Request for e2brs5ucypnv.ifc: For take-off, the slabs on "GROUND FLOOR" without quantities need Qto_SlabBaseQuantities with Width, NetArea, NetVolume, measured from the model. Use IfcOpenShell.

First a look at what the model holds.

```python
import ifcopenshell
import ifcopenshell.util.element
import ifcopenshell.util.unit

model = ifcopenshell.open("e2brs5ucypnv.ifc")
print(model.schema)
for unit_type in ("LENGTHUNIT", "AREAUNIT", "VOLUMEUNIT"):
    print(unit_type, ifcopenshell.util.unit.calculate_unit_scale(model, unit_type))
storey = next(s for s in model.by_type("IfcBuildingStorey") if s.Name == "GROUND FLOOR")
slabs = [e for e in ifcopenshell.util.element.get_decomposition(storey) if e.is_a("IfcSlab")]
for e in sorted(slabs, key=lambda e: e.id()):
    print(e.id(), e.is_a(), e.Name, list(ifcopenshell.util.element.get_psets(e, qtos_only=True)), sep=" | ")
```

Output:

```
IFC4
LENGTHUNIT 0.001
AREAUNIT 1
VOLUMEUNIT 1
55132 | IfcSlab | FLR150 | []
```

```python
import ifcopenshell
import ifcopenshell.api.pset
import ifcopenshell.geom
import ifcopenshell.util.element
import ifcopenshell.util.shape
import ifcopenshell.util.unit

model = ifcopenshell.open("e2brs5ucypnv.ifc")
unit_scale = ifcopenshell.util.unit.calculate_unit_scale(model)
area_scale = ifcopenshell.util.unit.calculate_unit_scale(model, "AREAUNIT")
volume_scale = ifcopenshell.util.unit.calculate_unit_scale(model, "VOLUMEUNIT")
settings = ifcopenshell.geom.settings()

storey = next(s for s in model.by_type("IfcBuildingStorey") if s.Name == "GROUND FLOOR")
slabs = [e for e in ifcopenshell.util.element.get_decomposition(storey) if e.is_a("IfcSlab")]

for e in sorted(slabs, key=lambda e: e.id()):
    if ifcopenshell.util.element.get_psets(e, qtos_only=True, should_inherit=False):
        continue
    # Geometry comes back in metres, in the element's own axes.
    shape = ifcopenshell.geom.create_shape(settings, e)
    values = {
        "Width": ifcopenshell.util.shape.get_z(shape.geometry) / unit_scale,
        "NetArea": ifcopenshell.util.shape.get_footprint_area(shape.geometry) / area_scale,
        "NetVolume": ifcopenshell.util.shape.get_volume(shape.geometry) / volume_scale,
    }
    qto = ifcopenshell.api.pset.add_qto(model, product=e, name="Qto_SlabBaseQuantities")
    ifcopenshell.api.pset.edit_qto(model, qto=qto, properties=values)
    print(e.id(), {k: round(v, 3) for k, v in values.items()})

model.write("e2brs5ucypnv_rev.ifc")
```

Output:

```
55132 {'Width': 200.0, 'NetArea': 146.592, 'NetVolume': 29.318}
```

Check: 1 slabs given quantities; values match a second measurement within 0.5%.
